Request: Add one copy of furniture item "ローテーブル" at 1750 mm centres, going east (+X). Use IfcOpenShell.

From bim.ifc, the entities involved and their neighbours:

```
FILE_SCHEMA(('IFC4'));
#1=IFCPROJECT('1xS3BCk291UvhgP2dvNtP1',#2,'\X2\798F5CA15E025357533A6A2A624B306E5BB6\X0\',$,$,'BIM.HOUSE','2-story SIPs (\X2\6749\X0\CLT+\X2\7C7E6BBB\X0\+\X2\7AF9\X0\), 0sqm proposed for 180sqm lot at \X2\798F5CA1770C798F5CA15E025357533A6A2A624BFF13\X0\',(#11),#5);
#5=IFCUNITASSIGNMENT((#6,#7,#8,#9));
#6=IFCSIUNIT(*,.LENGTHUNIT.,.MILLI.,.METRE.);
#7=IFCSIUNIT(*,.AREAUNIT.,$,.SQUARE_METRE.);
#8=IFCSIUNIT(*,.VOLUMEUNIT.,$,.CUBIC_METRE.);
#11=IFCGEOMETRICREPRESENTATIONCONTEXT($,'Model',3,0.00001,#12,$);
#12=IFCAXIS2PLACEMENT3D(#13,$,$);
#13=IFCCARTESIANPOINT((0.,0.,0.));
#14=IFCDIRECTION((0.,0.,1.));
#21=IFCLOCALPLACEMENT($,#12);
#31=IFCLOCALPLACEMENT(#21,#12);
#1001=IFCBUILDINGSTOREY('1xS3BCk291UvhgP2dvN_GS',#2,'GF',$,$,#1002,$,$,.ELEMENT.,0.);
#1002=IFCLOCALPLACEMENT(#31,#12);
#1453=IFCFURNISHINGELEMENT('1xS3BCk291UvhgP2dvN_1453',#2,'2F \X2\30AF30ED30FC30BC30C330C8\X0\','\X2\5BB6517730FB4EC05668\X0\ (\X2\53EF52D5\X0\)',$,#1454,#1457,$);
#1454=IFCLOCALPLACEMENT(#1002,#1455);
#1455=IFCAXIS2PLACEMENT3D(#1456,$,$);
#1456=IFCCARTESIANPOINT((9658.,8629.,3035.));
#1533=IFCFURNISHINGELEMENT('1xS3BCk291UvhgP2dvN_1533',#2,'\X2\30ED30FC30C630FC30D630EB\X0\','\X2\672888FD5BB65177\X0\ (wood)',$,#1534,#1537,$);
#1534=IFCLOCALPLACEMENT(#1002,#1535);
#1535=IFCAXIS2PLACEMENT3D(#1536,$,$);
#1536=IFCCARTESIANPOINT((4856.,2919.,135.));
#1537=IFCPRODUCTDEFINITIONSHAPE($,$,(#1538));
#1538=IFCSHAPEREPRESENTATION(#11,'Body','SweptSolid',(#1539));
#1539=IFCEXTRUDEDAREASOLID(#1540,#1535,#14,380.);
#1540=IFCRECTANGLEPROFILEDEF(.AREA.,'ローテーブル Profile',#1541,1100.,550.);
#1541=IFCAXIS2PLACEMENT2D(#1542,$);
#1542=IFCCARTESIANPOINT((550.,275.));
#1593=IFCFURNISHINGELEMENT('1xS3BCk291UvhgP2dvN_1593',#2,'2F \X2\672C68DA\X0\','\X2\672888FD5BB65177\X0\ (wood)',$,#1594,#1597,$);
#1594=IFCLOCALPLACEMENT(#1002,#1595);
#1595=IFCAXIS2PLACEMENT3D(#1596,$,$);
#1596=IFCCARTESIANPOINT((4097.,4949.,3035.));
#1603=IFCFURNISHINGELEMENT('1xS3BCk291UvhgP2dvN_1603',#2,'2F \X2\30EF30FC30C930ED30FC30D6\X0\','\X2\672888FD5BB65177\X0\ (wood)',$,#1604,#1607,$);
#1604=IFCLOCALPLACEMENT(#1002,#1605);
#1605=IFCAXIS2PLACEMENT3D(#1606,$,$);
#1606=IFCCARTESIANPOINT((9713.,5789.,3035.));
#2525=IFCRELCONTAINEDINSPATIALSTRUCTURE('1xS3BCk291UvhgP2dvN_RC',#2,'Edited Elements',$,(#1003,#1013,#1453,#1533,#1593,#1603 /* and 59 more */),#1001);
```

```python
import numpy as np
import ifcopenshell
import ifcopenshell.api.geometry
import ifcopenshell.api.root
import ifcopenshell.util.element
import ifcopenshell.util.placement

model = ifcopenshell.open("bim.ifc")


def reuse_history(source, copy):
    """copy_class also copies each property set's owner history, people and application; keep the originals."""
    for rel in copy.IsDefinedBy:
        if rel.is_a("IfcRelDefinesByProperties") and (history := rel.RelatingPropertyDefinition.OwnerHistory):
            rel.RelatingPropertyDefinition.OwnerHistory = source.OwnerHistory
            ifcopenshell.util.element.remove_deep2(model, history)


source = model.by_guid("1xS3BCk291UvhgP2dvN_1533")
base = ifcopenshell.util.placement.get_local_placement(source.ObjectPlacement)
step = np.array([1.0, 0.0, 0.0]) * 1750.0

for i in range(1, 2):
    copy = ifcopenshell.api.root.copy_class(model, product=source)
    copy.Representation = ifcopenshell.util.element.copy_deep(
        model, source.Representation, exclude=["IfcGeometricRepresentationContext", "IfcRepresentationMap"]
    )
    reuse_history(source, copy)
    matrix = base.copy()
    matrix[:3, 3] += i * step
    print("added at", matrix[:3, 3].round(3) + 0.0)
    ifcopenshell.api.geometry.edit_object_placement(model, product=copy, matrix=matrix, is_si=False)

model.write("bim_v2.ifc")
```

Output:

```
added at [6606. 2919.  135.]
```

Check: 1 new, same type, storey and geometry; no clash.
